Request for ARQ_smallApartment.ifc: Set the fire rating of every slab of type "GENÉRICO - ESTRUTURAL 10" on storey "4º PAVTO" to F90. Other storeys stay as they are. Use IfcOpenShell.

First a look at what the model holds.

```python
import ifcopenshell
import ifcopenshell.util.element

model = ifcopenshell.open("ARQ_smallApartment.ifc")
print(model.schema)
storey = next(s for s in model.by_type("IfcBuildingStorey") if s.Name == "4º PAVTO")
slabs = [e for e in ifcopenshell.util.element.get_decomposition(storey) if e.is_a("IfcSlab")]
seen = {}
for e in slabs:
    element_type = ifcopenshell.util.element.get_type(e)
    key = (element_type.Name if element_type != e and element_type else None, ifcopenshell.util.element.get_pset(e, "Pset_SlabCommon", "FireRating"))
    seen[key] = seen.get(key, 0) + 1
for (name, value), count in sorted(seen.items(), key=str):
    print(count, "x", name, "|", value)
```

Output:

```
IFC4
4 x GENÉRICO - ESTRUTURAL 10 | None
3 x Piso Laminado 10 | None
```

```python
import ifcopenshell
import ifcopenshell.api.pset
import ifcopenshell.util.element

model = ifcopenshell.open("ARQ_smallApartment.ifc")

storey = next(s for s in model.by_type("IfcBuildingStorey") if s.Name == "4º PAVTO")
slabs = [e for e in ifcopenshell.util.element.get_decomposition(storey) if e.is_a("IfcSlab")]

count = 0
for e in slabs:
    element_type = ifcopenshell.util.element.get_type(e)
    if element_type in (None, e) or element_type.Name != "GENÉRICO - ESTRUTURAL 10":
        continue
    # add_pset returns the element's existing set when there is one.
    pset = ifcopenshell.api.pset.add_pset(model, product=e, name="Pset_SlabCommon")
    ifcopenshell.api.pset.edit_pset(model, pset=pset, properties={"FireRating": "F90"})
    count += 1

print(count, "slabs updated")

model.write("ARQ_smallApartment_v2.ifc")
```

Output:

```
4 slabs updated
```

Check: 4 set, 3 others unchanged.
